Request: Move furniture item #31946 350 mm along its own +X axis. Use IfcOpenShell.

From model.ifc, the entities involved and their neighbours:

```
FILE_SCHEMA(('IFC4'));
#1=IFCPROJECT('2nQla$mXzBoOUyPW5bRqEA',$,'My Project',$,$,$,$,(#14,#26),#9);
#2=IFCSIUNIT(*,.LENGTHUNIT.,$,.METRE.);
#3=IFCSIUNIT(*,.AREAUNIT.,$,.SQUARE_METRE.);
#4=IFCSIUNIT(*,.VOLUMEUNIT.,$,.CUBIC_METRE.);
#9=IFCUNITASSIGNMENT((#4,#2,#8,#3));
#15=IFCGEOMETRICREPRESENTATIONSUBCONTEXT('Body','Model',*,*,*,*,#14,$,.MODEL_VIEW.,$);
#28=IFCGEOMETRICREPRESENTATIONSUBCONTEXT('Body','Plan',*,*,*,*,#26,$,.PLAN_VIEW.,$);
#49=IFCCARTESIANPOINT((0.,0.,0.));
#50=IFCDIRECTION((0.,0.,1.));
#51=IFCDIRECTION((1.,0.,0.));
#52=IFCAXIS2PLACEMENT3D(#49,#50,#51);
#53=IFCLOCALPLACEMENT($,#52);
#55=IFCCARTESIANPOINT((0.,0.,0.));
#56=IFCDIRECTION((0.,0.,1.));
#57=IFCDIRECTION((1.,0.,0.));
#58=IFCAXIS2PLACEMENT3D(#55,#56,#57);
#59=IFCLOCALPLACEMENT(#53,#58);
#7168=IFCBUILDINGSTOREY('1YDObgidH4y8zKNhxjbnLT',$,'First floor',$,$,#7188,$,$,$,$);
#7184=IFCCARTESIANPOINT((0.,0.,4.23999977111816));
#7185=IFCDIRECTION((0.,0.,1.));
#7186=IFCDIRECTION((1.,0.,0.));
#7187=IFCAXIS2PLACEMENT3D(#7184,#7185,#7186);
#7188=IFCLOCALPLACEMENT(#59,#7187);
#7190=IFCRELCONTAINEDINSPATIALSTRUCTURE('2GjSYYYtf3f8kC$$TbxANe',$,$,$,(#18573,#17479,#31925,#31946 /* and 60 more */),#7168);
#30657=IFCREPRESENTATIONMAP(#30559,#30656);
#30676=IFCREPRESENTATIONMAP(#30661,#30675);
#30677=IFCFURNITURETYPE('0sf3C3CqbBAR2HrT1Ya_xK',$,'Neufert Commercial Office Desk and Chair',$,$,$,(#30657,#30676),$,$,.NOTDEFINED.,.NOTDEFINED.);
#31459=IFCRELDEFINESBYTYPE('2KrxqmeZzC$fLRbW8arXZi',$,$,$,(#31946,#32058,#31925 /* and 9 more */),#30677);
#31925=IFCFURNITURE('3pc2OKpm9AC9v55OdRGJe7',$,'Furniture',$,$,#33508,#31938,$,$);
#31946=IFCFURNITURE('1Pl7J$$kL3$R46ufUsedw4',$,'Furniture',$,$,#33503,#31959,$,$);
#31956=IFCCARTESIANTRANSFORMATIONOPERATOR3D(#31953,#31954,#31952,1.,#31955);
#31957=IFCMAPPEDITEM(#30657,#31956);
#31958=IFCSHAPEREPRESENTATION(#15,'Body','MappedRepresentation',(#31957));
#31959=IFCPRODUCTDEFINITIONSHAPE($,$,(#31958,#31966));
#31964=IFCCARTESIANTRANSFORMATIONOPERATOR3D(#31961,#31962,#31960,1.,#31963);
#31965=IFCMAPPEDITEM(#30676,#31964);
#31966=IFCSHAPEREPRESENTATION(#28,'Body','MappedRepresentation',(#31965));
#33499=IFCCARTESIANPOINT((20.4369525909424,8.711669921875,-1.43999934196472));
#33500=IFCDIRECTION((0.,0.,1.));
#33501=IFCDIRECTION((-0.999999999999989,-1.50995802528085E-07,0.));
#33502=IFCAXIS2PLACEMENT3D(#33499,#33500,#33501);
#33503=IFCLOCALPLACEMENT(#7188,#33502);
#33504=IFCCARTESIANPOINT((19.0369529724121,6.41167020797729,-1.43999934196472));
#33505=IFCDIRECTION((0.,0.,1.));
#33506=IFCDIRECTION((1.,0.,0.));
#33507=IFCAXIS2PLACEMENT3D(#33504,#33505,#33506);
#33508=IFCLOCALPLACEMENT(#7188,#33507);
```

```python
import ifcopenshell
import ifcopenshell.api.geometry
import ifcopenshell.util.placement

model = ifcopenshell.open("model.ifc")

item = model.by_guid("1Pl7J$$kL3$R46ufUsedw4")
matrix = ifcopenshell.util.placement.get_local_placement(item.ObjectPlacement)
matrix[:3, 3] += matrix[:3, 0] * 0.35
ifcopenshell.api.geometry.edit_object_placement(model, product=item, matrix=matrix, is_si=False)

print(ifcopenshell.util.placement.get_local_placement(item.ObjectPlacement).round(3) + 0.0)

model.write("model_updated.ifc")
```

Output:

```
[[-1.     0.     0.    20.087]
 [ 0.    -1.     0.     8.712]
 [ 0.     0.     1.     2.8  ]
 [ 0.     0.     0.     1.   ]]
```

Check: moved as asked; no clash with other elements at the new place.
